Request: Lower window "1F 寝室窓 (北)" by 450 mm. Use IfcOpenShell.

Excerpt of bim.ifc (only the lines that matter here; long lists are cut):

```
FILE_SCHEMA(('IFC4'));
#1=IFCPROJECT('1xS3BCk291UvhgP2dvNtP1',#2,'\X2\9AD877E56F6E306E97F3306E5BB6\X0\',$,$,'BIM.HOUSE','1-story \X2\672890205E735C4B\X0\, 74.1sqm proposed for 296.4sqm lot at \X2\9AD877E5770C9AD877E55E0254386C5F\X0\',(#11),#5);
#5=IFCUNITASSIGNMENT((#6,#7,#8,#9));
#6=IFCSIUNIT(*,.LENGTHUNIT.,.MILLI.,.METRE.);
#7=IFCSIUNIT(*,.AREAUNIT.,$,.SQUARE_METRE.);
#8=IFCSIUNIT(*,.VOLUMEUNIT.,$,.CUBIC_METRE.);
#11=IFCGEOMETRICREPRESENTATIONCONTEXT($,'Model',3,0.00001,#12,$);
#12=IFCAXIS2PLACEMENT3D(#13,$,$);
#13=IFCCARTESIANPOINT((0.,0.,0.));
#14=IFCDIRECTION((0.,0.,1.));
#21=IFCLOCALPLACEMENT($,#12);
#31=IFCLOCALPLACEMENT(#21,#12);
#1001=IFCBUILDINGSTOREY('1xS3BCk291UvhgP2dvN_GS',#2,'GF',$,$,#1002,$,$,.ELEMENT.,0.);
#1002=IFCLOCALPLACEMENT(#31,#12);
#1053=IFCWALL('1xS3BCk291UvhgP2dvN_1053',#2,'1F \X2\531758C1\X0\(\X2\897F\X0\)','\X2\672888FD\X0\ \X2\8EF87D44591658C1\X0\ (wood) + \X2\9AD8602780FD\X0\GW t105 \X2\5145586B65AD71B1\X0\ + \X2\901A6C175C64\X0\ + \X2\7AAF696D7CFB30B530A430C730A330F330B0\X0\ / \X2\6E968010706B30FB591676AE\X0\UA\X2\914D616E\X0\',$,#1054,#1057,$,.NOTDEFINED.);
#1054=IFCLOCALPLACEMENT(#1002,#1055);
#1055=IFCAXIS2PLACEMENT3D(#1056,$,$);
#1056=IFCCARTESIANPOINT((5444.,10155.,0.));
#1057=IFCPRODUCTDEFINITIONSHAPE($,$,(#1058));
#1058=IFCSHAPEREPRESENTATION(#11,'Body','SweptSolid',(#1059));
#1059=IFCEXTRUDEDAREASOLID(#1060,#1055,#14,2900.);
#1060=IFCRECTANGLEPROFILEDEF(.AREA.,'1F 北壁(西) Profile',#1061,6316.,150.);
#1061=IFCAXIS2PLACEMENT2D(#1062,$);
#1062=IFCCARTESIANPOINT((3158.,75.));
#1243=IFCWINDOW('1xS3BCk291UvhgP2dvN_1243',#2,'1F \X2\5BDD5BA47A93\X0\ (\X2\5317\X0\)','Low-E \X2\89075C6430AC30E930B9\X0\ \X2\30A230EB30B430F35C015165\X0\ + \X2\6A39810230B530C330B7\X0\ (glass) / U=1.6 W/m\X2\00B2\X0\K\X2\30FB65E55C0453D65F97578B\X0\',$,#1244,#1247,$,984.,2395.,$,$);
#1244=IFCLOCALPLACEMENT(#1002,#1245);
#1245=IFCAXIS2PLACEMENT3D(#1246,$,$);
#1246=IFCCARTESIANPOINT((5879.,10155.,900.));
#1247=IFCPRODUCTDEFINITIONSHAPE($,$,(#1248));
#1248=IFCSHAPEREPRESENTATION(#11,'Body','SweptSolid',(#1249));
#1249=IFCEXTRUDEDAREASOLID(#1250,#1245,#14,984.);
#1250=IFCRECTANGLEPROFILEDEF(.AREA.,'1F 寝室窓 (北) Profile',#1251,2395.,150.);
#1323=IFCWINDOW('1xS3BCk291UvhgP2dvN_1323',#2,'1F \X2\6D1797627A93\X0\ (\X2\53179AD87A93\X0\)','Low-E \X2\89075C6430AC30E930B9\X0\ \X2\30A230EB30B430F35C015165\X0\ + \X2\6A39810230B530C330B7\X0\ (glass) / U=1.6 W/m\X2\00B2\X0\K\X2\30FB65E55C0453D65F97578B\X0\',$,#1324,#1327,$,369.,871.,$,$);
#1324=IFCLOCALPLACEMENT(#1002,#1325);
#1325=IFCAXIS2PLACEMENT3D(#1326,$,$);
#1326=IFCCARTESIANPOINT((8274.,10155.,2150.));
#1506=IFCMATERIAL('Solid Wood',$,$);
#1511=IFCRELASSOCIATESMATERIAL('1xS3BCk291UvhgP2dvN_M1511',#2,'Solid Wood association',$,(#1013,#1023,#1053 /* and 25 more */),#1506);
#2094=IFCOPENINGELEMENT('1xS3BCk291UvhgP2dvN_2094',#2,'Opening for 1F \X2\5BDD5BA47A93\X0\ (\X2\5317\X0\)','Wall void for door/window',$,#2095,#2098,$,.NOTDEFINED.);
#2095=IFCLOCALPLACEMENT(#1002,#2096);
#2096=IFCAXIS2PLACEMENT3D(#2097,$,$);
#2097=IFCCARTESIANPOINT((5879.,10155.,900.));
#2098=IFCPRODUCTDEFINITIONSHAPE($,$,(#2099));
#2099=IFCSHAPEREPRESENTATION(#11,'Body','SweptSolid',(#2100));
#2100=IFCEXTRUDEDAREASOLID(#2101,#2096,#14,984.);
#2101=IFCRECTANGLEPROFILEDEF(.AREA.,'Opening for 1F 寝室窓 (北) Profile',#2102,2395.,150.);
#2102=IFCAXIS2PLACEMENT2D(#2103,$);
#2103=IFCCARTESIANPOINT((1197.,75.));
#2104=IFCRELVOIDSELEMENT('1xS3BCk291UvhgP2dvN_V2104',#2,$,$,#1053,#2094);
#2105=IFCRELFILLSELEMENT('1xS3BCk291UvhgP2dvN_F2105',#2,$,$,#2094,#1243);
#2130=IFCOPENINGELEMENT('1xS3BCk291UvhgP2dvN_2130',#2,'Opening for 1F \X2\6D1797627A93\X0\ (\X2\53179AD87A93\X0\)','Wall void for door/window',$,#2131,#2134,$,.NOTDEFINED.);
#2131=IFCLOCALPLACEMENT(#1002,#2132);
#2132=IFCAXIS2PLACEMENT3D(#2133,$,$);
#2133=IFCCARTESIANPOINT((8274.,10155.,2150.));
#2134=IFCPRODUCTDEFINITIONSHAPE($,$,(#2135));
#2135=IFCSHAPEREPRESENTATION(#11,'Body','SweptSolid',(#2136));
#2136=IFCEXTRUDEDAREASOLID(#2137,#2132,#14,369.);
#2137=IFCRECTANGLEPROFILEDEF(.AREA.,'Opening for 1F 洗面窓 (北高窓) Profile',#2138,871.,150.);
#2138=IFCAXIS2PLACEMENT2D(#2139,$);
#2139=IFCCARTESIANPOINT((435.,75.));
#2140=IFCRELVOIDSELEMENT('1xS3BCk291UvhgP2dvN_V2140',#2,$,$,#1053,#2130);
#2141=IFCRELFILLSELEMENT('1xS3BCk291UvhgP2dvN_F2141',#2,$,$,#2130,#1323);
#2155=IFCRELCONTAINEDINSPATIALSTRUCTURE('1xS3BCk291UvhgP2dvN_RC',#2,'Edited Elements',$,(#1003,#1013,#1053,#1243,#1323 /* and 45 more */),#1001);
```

```python
import numpy as np
import ifcopenshell
import ifcopenshell.api.geometry
import ifcopenshell.util.placement
import ifcopenshell.util.unit

model = ifcopenshell.open("bim.ifc")
unit_scale = ifcopenshell.util.unit.calculate_unit_scale(model)

window = model.by_guid("1xS3BCk291UvhgP2dvN_1243")
opening = window.FillsVoids[0].RelatingOpeningElement
dz = -0.45 / unit_scale

shift = np.array([0.0, 0.0, dz])
# The window is not placed relative to its opening, so move both.
for product in (opening, window):
    matrix = ifcopenshell.util.placement.get_local_placement(product.ObjectPlacement)
    matrix[:3, 3] += shift
    ifcopenshell.api.geometry.edit_object_placement(model, product=product, matrix=matrix, is_si=False)

print(f"moved by {dz * unit_scale:+.3f} m")

model.write("bim_edited.ifc")
```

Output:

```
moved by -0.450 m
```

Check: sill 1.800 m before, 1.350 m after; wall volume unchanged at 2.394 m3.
